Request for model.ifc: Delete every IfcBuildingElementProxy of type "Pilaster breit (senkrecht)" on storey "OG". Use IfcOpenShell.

First a look at what the model holds.

```python
import ifcopenshell
import ifcopenshell.util.element

model = ifcopenshell.open("model.ifc")
print(model.schema)
storey = next(s for s in model.by_type("IfcBuildingStorey") if s.Name == "OG")
proxies = [e for e in ifcopenshell.util.element.get_decomposition(storey) if e.is_a("IfcBuildingElementProxy")]
seen = {}
for e in proxies:
    element_type = ifcopenshell.util.element.get_type(e)
    name = element_type.Name if element_type not in (None, e) else None
    seen[name] = seen.get(name, 0) + 1
for name, count in sorted(seen.items(), key=str):
    print(count, "x", name)
```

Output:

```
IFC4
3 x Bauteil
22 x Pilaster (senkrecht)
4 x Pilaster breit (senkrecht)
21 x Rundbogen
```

```python
import ifcopenshell
import ifcopenshell.api.root
import ifcopenshell.util.element

model = ifcopenshell.open("model.ifc")

storey = next(s for s in model.by_type("IfcBuildingStorey") if s.Name == "OG")
proxies = [e for e in ifcopenshell.util.element.get_decomposition(storey) if e.is_a("IfcBuildingElementProxy")]
targets = [e for e in proxies if (t := ifcopenshell.util.element.get_type(e)) not in (None, e) and t.Name == "Pilaster breit (senkrecht)"]

for e in targets:
    ifcopenshell.api.root.remove_product(model, product=e)
print(len(targets), "removed")

model.write("model-out.ifc")
```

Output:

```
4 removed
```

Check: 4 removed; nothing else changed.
